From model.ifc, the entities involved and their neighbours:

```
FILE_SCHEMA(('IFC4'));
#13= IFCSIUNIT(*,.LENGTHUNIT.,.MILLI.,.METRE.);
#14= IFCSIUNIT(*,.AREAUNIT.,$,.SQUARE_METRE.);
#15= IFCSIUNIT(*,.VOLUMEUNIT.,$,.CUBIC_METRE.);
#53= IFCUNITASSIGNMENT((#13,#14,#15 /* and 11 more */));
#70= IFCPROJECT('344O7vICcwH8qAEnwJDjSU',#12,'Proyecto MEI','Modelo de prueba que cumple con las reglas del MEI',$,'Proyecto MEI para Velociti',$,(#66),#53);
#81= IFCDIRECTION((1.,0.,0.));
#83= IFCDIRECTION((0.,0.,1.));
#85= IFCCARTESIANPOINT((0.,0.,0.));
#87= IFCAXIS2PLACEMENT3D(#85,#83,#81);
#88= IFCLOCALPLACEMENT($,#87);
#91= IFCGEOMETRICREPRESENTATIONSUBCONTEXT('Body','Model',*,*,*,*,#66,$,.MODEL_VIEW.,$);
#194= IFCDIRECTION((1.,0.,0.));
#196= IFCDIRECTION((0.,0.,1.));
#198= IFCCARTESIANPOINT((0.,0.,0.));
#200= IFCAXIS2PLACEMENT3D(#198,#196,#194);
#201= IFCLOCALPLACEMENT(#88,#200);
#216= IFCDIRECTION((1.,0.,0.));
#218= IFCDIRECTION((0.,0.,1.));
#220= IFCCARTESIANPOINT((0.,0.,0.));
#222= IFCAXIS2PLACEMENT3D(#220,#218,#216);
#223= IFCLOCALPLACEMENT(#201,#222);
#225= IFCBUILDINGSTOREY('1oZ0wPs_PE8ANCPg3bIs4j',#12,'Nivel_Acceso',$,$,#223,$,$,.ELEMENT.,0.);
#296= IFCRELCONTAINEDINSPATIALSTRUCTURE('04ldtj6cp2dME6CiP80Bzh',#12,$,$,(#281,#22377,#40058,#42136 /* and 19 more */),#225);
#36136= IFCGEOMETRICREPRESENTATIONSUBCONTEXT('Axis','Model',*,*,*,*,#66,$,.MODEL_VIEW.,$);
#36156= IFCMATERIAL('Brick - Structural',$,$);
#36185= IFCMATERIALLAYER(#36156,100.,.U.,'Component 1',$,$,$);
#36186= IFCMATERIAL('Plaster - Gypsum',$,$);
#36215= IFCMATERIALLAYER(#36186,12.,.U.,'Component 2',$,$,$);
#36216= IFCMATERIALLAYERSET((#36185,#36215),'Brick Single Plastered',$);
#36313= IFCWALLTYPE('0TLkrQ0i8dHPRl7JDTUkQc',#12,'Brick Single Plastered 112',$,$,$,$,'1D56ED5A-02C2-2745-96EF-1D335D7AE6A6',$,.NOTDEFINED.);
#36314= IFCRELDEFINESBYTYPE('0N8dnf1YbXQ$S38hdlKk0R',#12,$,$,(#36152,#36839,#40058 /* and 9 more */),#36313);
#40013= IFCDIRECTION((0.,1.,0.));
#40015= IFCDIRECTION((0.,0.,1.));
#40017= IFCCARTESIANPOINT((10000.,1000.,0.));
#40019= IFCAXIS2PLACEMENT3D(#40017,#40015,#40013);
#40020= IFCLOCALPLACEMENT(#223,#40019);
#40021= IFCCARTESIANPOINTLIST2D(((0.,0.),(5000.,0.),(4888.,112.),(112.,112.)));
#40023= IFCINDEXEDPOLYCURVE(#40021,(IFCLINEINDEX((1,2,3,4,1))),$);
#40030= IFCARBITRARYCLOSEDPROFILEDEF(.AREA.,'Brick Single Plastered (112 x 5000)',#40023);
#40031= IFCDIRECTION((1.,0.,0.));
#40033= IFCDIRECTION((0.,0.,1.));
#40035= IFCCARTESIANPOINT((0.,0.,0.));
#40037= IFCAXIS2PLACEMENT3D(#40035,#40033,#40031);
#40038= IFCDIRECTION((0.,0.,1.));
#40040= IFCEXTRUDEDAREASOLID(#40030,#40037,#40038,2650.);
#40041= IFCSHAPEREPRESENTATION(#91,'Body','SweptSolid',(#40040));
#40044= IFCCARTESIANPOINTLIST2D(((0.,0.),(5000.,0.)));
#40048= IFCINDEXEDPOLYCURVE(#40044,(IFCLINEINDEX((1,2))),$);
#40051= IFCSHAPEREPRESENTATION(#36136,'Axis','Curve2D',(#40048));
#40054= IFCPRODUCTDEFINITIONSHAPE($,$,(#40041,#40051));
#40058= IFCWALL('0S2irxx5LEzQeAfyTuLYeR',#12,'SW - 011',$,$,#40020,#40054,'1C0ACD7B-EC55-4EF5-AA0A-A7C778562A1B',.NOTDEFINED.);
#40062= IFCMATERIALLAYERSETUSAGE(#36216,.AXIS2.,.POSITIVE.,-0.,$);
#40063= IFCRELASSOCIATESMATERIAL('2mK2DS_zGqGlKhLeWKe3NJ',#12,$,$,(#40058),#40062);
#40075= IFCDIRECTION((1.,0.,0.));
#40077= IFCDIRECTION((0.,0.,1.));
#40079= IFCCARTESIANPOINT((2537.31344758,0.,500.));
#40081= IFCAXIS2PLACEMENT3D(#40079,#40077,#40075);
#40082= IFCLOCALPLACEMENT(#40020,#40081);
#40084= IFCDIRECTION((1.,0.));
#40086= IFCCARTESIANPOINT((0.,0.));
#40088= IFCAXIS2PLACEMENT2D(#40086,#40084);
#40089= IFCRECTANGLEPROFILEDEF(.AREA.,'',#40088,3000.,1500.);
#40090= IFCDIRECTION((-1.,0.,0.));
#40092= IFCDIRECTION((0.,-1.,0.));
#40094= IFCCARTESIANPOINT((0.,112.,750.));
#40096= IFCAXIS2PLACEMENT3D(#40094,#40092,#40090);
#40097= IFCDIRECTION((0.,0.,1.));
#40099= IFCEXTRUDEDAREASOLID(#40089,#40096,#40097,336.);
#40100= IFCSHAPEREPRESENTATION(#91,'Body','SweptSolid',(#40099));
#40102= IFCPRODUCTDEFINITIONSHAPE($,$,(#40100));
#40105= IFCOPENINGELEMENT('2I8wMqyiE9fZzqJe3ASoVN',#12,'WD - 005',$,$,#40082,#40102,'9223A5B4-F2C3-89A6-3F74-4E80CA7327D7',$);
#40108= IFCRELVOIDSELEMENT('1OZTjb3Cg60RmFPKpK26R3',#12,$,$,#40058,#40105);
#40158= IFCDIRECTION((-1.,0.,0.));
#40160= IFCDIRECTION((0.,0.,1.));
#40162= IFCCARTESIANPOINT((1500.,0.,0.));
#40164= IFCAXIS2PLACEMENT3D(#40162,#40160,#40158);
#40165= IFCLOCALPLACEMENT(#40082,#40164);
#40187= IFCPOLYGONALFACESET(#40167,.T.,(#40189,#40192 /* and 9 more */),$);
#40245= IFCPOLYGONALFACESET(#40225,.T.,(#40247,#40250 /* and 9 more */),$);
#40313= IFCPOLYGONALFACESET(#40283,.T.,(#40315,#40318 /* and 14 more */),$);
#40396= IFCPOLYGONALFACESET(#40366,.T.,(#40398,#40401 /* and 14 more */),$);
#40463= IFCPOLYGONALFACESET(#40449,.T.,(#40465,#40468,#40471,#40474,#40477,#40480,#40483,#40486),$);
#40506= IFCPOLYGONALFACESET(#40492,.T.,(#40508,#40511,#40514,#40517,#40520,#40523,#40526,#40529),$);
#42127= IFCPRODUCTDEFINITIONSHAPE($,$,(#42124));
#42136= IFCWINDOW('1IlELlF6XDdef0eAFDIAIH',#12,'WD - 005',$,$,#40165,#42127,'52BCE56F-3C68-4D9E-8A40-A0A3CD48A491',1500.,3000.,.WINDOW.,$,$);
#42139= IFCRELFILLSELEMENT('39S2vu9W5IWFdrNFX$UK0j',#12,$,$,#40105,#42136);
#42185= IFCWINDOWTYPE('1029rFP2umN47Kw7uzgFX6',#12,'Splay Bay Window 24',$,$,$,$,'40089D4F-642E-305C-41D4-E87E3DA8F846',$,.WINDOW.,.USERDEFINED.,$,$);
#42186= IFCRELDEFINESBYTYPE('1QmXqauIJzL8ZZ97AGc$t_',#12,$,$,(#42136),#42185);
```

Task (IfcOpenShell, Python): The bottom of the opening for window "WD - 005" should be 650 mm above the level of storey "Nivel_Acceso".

```python
import numpy as np
import ifcopenshell
import ifcopenshell.api.geometry
import ifcopenshell.geom
import ifcopenshell.util.element
import ifcopenshell.util.placement
import ifcopenshell.util.shape
import ifcopenshell.util.unit

model = ifcopenshell.open("model.ifc")
unit_scale = ifcopenshell.util.unit.calculate_unit_scale(model)

window = model.by_guid("1IlELlF6XDdef0eAFDIAIH")
opening = window.FillsVoids[0].RelatingOpeningElement
storey = ifcopenshell.util.element.get_container(window, ifc_class="IfcBuildingStorey")
level = ifcopenshell.util.placement.get_local_placement(storey.ObjectPlacement)[2, 3]

# The opening's origin need not be at the sill, so measure its lowest point.
shape = ifcopenshell.geom.create_shape(ifcopenshell.geom.settings(), opening)
bottom = ifcopenshell.util.shape.get_shape_bottom_elevation(shape, shape.geometry) / unit_scale
dz = level + 650.0 - bottom

shift = np.array([0.0, 0.0, dz])
# The window is placed relative to its opening, so it follows when the opening moves.
matrix = ifcopenshell.util.placement.get_local_placement(opening.ObjectPlacement)
matrix[:3, 3] += shift
ifcopenshell.api.geometry.edit_object_placement(
    model, product=opening, matrix=matrix, is_si=False, should_transform_children=True
)

print(f"moved by {dz * unit_scale:+.3f} m")

model.write("model_v2.ifc")
```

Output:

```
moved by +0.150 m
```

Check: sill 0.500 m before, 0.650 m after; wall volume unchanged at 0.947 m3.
